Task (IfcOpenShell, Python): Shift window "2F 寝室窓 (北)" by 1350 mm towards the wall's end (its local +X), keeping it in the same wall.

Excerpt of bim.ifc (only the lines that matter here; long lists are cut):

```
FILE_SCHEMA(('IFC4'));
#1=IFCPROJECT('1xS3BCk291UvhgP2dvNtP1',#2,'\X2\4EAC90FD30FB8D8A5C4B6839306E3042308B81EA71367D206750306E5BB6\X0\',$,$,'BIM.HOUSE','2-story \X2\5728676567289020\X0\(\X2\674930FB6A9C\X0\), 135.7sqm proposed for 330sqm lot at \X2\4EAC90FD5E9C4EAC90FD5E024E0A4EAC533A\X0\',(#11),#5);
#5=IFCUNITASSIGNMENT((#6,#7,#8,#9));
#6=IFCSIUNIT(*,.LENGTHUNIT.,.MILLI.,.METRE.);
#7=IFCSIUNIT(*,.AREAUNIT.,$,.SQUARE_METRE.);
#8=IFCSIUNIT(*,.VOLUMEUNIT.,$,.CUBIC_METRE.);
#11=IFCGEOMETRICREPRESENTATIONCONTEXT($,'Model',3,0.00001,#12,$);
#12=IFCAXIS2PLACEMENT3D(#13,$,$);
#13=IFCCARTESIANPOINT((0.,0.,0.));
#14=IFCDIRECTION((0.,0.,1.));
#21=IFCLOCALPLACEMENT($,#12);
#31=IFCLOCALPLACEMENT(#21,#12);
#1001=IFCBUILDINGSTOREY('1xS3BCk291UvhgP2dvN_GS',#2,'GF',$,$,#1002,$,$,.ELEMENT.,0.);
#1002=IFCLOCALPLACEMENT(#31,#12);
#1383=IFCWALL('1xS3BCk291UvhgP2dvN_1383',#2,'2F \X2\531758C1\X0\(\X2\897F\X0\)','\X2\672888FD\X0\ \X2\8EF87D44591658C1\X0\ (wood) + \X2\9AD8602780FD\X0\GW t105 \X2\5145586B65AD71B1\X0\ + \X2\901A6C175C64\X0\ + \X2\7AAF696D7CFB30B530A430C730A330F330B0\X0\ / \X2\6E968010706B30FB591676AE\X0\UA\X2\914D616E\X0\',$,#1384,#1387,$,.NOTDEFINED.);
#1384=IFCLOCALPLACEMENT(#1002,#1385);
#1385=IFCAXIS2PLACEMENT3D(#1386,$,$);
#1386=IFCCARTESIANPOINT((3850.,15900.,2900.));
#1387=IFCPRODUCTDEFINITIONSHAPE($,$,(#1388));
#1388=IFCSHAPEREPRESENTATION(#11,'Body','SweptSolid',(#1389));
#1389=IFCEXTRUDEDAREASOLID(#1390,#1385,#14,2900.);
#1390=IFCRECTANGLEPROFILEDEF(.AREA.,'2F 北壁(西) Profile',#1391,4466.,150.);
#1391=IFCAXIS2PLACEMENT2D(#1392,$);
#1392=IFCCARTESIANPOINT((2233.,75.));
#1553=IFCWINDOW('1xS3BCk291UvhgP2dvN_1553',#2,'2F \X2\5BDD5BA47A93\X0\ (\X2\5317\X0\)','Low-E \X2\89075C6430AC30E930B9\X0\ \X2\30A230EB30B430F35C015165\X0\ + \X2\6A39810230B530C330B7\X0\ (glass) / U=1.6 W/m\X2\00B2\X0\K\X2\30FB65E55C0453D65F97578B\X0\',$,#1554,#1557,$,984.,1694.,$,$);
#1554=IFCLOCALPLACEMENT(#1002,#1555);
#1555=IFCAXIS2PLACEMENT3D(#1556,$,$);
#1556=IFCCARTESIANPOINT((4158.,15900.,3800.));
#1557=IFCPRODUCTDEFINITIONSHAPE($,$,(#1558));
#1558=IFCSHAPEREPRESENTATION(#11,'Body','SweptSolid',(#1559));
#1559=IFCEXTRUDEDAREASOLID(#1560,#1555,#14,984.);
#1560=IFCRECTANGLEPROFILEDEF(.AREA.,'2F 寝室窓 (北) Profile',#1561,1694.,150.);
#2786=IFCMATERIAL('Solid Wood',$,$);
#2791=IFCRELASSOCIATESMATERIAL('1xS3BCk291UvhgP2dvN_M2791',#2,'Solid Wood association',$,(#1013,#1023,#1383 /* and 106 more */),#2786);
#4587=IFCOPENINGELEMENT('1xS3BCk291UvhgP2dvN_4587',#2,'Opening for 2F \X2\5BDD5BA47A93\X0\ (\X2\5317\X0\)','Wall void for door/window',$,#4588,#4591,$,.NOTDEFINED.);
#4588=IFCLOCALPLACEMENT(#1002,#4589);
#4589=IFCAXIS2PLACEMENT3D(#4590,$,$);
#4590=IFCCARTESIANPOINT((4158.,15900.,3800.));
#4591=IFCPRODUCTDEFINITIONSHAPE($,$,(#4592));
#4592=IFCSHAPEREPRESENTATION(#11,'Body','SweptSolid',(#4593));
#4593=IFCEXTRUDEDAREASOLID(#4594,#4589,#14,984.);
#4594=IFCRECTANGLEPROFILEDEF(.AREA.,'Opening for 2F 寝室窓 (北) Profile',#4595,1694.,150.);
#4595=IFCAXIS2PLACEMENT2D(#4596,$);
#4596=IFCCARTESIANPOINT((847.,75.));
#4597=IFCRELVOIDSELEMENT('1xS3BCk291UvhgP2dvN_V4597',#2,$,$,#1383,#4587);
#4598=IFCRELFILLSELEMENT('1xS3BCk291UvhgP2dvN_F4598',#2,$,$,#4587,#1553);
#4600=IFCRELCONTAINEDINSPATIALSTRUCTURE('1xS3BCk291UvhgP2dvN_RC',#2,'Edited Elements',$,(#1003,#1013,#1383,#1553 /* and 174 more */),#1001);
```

```python
import ifcopenshell
import ifcopenshell.api.geometry
import ifcopenshell.util.placement

model = ifcopenshell.open("bim.ifc")

window = model.by_id(1553)
opening = window.FillsVoids[0].RelatingOpeningElement
wall = opening.VoidsElements[0].RelatingBuildingElement

wall_matrix = ifcopenshell.util.placement.get_local_placement(wall.ObjectPlacement)
shift = wall_matrix[:3, 0] * 1350.0
before = ifcopenshell.util.placement.get_local_placement(window.ObjectPlacement)[:3, 3].copy()

# The window is not placed relative to its opening, so move both.
for product in (opening, window):
    matrix = ifcopenshell.util.placement.get_local_placement(product.ObjectPlacement)
    matrix[:3, 3] += shift
    ifcopenshell.api.geometry.edit_object_placement(model, product=product, matrix=matrix, is_si=False)

after = ifcopenshell.util.placement.get_local_placement(window.ObjectPlacement)[:3, 3]
print("window moved by", (after - before).round(3) + 0.0)

model.write("bim_rev.ifc")
```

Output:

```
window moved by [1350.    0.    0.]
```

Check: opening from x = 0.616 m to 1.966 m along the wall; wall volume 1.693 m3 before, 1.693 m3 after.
